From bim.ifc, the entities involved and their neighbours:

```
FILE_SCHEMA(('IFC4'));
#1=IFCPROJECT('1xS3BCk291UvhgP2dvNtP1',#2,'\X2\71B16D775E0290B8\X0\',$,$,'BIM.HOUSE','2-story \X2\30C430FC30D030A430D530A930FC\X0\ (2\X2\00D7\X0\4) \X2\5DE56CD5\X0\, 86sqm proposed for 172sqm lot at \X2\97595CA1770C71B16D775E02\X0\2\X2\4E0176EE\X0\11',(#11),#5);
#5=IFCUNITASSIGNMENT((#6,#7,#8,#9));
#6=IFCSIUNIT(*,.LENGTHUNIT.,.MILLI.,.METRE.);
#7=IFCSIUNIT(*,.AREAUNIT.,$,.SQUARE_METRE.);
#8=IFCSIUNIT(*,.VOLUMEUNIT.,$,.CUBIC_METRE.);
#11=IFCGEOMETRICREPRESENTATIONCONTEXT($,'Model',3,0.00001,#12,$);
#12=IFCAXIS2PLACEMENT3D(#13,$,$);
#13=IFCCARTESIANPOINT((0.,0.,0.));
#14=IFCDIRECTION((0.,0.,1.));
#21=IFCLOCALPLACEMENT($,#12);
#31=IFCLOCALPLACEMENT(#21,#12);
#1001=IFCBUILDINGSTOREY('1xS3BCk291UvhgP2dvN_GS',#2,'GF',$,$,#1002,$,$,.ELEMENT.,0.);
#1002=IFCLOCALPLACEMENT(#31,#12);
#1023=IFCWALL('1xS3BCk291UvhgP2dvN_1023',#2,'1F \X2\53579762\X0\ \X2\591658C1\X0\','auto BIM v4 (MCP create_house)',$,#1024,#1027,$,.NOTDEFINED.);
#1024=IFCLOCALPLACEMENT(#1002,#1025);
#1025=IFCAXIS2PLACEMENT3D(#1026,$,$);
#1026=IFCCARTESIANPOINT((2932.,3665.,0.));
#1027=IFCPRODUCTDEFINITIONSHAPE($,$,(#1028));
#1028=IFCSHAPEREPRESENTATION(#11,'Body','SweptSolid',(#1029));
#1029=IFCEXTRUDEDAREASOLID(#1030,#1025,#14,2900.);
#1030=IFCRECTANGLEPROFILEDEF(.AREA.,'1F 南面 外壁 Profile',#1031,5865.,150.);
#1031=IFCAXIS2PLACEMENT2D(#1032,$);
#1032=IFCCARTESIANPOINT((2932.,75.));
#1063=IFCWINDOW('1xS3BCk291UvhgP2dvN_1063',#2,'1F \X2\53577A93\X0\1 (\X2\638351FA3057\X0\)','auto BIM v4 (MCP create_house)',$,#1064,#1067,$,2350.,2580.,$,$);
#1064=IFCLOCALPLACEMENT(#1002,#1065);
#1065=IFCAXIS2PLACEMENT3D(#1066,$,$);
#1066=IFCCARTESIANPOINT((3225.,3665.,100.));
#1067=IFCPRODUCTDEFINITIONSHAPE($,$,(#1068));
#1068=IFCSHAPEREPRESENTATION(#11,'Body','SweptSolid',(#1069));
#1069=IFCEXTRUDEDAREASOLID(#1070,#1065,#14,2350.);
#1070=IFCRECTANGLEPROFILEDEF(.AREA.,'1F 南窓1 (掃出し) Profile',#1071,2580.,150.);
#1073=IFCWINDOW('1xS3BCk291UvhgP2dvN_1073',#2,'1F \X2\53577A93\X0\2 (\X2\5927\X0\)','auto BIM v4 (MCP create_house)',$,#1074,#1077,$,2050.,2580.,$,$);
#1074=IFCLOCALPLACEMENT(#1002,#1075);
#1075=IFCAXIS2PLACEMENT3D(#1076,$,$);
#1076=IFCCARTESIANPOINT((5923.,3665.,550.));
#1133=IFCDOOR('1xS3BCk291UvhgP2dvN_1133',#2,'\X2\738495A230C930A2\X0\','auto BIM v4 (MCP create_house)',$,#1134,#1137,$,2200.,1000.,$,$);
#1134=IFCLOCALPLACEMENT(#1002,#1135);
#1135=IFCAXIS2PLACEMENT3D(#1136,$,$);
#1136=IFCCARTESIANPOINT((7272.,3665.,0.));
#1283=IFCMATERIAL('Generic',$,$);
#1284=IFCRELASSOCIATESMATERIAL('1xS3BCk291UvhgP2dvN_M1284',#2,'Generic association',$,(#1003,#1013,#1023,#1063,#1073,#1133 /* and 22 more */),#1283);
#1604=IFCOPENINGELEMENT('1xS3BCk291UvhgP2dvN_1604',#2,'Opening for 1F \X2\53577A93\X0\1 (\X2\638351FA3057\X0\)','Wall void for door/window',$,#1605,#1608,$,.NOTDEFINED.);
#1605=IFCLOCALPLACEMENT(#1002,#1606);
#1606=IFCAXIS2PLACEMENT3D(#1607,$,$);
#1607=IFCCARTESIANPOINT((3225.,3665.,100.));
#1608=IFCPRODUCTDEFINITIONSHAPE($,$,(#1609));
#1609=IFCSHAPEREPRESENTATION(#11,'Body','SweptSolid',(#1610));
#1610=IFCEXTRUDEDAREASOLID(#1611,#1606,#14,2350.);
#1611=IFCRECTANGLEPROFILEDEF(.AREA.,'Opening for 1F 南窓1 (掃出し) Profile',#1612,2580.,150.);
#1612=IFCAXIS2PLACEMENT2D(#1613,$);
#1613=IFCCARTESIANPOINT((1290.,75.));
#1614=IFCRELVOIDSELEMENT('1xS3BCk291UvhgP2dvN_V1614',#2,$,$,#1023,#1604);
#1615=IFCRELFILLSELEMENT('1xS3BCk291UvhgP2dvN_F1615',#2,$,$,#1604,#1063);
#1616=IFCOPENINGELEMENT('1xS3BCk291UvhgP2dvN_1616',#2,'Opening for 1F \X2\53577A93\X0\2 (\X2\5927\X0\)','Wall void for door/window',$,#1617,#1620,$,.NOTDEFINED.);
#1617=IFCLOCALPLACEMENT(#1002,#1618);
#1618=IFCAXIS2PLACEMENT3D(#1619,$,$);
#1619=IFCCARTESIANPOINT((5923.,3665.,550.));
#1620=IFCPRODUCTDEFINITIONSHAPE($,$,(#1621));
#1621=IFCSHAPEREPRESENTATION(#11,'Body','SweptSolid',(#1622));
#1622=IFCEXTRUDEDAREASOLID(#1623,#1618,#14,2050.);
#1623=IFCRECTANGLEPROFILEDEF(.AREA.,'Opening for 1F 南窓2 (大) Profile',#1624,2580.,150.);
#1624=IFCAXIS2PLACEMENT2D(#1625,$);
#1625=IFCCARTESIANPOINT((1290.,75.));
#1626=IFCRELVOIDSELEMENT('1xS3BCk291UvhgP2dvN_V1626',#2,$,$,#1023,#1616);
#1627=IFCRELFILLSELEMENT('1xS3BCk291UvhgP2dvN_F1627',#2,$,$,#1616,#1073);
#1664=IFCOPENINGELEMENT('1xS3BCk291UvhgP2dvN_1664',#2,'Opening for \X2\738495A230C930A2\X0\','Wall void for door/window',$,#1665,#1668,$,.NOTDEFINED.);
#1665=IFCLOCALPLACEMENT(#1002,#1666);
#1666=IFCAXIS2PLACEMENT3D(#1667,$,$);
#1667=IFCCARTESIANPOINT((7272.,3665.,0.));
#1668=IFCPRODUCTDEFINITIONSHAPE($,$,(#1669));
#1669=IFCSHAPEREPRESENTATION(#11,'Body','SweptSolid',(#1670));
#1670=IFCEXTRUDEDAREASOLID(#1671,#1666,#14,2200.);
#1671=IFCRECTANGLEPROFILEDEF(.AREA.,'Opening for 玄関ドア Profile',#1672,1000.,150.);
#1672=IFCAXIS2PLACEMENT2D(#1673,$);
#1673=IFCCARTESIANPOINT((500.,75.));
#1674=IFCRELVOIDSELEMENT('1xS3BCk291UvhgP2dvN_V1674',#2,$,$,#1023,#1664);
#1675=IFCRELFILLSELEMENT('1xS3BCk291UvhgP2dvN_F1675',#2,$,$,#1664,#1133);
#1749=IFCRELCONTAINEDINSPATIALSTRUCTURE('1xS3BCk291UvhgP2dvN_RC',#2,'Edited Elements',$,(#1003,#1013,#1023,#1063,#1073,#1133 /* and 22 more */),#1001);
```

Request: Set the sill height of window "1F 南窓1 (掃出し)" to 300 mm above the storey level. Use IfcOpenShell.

```python
import numpy as np
import ifcopenshell
import ifcopenshell.api.geometry
import ifcopenshell.geom
import ifcopenshell.util.element
import ifcopenshell.util.placement
import ifcopenshell.util.shape
import ifcopenshell.util.unit

model = ifcopenshell.open("bim.ifc")
unit_scale = ifcopenshell.util.unit.calculate_unit_scale(model)

window = model.by_guid("1xS3BCk291UvhgP2dvN_1063")
opening = window.FillsVoids[0].RelatingOpeningElement
storey = ifcopenshell.util.element.get_container(window, ifc_class="IfcBuildingStorey")
level = ifcopenshell.util.placement.get_local_placement(storey.ObjectPlacement)[2, 3]

# The opening's origin need not be at the sill, so measure its lowest point.
shape = ifcopenshell.geom.create_shape(ifcopenshell.geom.settings(), opening)
bottom = ifcopenshell.util.shape.get_shape_bottom_elevation(shape, shape.geometry) / unit_scale
dz = level + 300.0 - bottom

shift = np.array([0.0, 0.0, dz])
# The window is not placed relative to its opening, so move both.
for product in (opening, window):
    matrix = ifcopenshell.util.placement.get_local_placement(product.ObjectPlacement)
    matrix[:3, 3] += shift
    ifcopenshell.api.geometry.edit_object_placement(model, product=product, matrix=matrix, is_si=False)

print(f"moved by {dz * unit_scale:+.3f} m")

model.write("bim_updated.ifc")
```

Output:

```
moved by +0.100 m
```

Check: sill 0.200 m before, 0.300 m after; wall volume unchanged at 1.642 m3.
